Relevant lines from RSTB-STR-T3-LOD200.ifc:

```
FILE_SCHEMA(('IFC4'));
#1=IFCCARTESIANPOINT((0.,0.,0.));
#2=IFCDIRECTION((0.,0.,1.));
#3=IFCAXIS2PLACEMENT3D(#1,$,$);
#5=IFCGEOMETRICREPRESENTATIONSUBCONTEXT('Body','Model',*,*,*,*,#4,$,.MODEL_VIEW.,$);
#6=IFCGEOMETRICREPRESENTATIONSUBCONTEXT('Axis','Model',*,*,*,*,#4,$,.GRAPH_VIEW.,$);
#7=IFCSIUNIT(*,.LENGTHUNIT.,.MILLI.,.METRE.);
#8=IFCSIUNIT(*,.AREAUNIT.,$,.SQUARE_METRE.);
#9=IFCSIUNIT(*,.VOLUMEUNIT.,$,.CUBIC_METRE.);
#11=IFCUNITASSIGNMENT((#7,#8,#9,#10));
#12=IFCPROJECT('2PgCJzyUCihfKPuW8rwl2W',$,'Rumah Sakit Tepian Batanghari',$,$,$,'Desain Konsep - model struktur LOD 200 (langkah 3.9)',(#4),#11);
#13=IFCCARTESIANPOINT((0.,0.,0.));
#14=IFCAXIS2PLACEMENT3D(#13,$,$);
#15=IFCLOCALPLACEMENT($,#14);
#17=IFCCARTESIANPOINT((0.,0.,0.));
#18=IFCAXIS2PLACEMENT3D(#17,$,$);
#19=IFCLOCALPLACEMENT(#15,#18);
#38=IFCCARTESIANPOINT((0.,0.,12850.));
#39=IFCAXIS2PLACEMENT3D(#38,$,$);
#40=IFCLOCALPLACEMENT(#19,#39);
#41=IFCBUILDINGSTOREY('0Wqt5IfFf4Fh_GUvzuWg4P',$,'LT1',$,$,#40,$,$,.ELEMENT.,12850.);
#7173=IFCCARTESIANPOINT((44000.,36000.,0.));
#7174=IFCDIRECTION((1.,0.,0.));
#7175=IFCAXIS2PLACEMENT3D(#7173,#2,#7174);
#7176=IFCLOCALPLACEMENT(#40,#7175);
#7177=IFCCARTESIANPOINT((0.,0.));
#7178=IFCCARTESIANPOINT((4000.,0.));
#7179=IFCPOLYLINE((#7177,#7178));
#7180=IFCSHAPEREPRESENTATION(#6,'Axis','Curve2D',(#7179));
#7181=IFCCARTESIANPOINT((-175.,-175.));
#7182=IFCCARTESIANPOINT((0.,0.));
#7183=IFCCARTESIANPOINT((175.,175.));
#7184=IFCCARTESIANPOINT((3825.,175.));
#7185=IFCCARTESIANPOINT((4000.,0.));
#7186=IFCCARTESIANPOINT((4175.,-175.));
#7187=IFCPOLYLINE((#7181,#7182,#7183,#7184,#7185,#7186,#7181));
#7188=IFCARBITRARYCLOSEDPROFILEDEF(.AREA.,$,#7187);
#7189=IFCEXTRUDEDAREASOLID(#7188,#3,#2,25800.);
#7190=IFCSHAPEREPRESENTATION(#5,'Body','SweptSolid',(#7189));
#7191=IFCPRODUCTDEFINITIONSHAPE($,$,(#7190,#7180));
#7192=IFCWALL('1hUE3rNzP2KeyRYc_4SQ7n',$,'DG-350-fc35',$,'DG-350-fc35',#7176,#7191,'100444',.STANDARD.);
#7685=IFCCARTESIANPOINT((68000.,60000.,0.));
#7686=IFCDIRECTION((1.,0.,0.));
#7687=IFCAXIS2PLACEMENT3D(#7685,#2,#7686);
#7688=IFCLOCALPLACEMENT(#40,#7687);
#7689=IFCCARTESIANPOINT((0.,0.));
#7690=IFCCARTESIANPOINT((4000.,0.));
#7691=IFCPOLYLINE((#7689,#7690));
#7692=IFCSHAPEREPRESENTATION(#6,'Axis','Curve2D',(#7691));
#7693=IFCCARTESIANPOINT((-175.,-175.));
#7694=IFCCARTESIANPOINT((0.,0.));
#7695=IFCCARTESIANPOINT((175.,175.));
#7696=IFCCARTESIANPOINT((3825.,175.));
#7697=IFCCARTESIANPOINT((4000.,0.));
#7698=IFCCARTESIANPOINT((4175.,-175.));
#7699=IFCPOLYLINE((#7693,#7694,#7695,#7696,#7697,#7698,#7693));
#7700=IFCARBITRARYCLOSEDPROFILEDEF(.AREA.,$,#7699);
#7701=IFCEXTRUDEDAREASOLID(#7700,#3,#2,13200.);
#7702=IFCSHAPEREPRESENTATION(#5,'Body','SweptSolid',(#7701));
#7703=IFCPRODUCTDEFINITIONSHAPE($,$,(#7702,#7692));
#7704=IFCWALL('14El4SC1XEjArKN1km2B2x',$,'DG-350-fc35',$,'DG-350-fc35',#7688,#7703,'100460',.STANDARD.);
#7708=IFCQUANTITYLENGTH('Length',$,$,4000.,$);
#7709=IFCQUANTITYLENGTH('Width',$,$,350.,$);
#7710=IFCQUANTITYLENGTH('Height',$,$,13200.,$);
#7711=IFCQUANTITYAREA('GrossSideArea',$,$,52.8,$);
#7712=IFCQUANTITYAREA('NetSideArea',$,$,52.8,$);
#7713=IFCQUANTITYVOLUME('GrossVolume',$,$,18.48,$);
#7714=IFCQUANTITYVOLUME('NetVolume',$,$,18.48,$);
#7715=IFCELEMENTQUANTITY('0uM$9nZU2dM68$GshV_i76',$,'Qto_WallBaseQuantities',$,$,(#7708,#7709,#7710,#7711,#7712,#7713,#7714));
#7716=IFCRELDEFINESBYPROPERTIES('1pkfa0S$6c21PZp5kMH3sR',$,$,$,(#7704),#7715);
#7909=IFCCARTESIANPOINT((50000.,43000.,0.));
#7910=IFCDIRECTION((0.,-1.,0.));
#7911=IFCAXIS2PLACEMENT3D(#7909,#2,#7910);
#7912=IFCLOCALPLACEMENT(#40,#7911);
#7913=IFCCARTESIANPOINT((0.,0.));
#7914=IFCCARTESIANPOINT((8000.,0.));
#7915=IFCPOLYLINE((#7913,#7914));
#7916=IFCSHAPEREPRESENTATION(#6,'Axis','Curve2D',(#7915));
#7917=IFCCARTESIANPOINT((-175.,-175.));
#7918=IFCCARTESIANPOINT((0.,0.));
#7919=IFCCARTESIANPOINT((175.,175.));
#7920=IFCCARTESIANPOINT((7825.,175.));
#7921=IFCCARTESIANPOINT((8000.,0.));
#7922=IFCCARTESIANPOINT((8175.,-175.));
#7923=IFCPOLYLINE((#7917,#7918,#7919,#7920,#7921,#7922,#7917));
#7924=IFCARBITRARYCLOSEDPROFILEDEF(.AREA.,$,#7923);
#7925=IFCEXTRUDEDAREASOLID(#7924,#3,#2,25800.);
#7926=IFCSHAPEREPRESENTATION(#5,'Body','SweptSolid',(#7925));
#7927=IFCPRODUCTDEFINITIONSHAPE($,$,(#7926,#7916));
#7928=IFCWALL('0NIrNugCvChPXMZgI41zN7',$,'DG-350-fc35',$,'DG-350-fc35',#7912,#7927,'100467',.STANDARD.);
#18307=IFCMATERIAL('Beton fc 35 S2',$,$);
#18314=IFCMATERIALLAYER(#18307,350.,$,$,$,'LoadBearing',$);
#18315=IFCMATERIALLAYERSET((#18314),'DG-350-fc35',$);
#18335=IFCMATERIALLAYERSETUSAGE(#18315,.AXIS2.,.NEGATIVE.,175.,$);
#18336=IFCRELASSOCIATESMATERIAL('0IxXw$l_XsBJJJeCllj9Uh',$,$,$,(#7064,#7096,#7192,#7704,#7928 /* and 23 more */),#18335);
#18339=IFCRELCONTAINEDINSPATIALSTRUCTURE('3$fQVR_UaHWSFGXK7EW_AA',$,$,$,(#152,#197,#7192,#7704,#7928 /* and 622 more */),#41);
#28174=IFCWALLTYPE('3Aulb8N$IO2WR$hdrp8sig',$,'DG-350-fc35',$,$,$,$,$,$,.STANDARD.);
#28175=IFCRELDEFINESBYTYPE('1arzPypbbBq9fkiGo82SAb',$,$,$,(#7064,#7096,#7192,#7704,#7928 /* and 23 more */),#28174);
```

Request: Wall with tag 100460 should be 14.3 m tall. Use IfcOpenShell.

```python
import ifcopenshell
import ifcopenshell.api.pset
import ifcopenshell.geom
import ifcopenshell.util.element
import ifcopenshell.util.representation
import ifcopenshell.util.shape
import ifcopenshell.util.unit

model = ifcopenshell.open("RSTB-STR-T3-LOD200.ifc")
unit_scale = ifcopenshell.util.unit.calculate_unit_scale(model)
area_scale = ifcopenshell.util.unit.calculate_unit_scale(model, "AREAUNIT")
volume_scale = ifcopenshell.util.unit.calculate_unit_scale(model, "VOLUMEUNIT")
settings = ifcopenshell.geom.settings()


def volume(element):
    """Net volume in cubic metres, openings subtracted."""
    shape = ifcopenshell.geom.create_shape(settings, element)
    return ifcopenshell.util.shape.get_volume(shape.geometry)


wall = model.by_guid("14El4SC1XEjArKN1km2B2x")
before = volume(wall)

body = ifcopenshell.util.representation.get_representation(wall, "Model", "Body")
solid = body.Items[0]
old_height = solid.Depth
solid.Depth = 14300.0
after = volume(wall)
thickness = 0.35  # wall thickness in metres

# Update the stored height, areas and volumes.
qto = model.by_id(ifcopenshell.util.element.get_pset(wall, "Qto_WallBaseQuantities", should_inherit=False)["id"])
ifcopenshell.api.pset.edit_qto(model, qto=qto, properties={
    "Height": solid.Depth,
    "GrossSideArea": ifcopenshell.util.element.get_pset(wall, "Qto_WallBaseQuantities", "GrossSideArea") * solid.Depth / old_height,
    "NetSideArea": after / thickness / area_scale,
    "GrossVolume": ifcopenshell.util.element.get_pset(wall, "Qto_WallBaseQuantities", "GrossVolume") * solid.Depth / old_height,
    "NetVolume": after / volume_scale,
})

print(f"height {old_height:g} -> {solid.Depth:g}, volume {before:.3f} -> {after:.3f} m3")

model.write("RSTB-STR-T3-LOD200-out.ifc")
```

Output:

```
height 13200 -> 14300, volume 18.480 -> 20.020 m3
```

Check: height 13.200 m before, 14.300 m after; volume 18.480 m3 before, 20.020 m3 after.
